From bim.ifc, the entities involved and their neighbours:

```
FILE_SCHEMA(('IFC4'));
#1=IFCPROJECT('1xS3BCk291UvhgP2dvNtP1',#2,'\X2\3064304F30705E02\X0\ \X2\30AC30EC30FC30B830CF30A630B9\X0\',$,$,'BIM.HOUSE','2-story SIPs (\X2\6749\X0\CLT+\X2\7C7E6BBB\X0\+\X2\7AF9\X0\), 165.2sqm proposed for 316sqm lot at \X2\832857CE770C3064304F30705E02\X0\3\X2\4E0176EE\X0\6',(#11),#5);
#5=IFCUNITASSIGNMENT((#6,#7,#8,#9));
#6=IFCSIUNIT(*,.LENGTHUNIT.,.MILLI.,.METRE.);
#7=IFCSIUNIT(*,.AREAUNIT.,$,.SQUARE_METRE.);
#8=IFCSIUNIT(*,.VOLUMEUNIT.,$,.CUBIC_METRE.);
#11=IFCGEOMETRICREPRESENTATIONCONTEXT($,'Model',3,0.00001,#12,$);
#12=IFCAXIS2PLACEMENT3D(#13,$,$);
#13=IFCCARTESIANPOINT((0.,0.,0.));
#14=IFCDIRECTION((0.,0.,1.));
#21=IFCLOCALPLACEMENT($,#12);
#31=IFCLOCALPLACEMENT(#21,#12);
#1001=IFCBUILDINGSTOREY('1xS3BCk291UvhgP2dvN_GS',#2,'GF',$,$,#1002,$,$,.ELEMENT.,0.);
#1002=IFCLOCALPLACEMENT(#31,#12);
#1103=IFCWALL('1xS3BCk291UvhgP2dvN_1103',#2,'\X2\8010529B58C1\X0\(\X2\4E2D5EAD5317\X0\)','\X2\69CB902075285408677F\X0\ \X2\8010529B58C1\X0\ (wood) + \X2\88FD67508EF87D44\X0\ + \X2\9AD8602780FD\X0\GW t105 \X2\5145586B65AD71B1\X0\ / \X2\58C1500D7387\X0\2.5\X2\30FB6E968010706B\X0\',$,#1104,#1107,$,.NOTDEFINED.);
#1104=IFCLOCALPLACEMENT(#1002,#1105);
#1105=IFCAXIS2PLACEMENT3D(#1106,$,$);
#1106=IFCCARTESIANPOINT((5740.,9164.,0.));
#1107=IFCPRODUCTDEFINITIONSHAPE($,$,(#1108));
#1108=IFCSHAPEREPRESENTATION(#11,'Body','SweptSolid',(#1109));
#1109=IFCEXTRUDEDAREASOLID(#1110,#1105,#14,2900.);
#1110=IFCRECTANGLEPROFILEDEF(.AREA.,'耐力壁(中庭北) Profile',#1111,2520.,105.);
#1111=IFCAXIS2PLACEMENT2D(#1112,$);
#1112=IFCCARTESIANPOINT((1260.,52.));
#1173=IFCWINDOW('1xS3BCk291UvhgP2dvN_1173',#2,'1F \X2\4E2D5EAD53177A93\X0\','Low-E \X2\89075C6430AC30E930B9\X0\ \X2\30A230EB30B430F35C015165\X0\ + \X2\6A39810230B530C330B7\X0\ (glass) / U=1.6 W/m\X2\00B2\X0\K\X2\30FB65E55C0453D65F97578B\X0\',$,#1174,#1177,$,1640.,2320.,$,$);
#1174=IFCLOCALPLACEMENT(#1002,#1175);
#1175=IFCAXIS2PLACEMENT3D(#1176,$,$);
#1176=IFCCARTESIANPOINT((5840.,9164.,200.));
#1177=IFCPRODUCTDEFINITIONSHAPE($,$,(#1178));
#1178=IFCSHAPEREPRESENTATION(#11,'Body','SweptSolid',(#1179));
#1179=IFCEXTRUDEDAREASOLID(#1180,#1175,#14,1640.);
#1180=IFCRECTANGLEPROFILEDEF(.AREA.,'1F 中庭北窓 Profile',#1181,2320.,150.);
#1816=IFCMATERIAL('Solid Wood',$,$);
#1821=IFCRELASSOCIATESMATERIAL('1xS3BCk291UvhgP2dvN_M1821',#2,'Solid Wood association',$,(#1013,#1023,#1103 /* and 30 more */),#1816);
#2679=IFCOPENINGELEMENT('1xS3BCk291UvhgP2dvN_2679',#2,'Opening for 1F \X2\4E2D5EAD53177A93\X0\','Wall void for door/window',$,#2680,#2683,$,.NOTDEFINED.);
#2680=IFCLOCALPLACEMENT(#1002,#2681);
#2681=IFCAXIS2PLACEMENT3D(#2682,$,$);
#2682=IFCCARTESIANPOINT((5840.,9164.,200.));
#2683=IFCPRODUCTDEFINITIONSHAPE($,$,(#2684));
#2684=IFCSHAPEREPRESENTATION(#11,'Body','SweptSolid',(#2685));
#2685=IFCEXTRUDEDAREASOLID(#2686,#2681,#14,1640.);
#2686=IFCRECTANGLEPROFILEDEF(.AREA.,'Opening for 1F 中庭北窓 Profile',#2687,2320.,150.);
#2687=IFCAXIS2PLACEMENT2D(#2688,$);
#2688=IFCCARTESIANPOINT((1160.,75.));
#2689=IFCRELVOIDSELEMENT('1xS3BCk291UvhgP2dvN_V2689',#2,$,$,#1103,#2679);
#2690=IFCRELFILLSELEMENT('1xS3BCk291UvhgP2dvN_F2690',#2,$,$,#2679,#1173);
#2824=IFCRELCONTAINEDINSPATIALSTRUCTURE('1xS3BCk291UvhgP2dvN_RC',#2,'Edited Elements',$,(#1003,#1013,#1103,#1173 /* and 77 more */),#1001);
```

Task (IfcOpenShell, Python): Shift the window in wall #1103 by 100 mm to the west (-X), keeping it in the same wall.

```python
import ifcopenshell
import ifcopenshell.api.geometry
import ifcopenshell.util.placement
import ifcopenshell.util.unit

model = ifcopenshell.open("bim.ifc")
unit_scale = ifcopenshell.util.unit.calculate_unit_scale(model)

window = model.by_guid("1xS3BCk291UvhgP2dvN_1173")
opening = window.FillsVoids[0].RelatingOpeningElement
wall = opening.VoidsElements[0].RelatingBuildingElement

wall_matrix = ifcopenshell.util.placement.get_local_placement(wall.ObjectPlacement)
shift = wall_matrix[:3, 0] * -0.1 / unit_scale
before = ifcopenshell.util.placement.get_local_placement(window.ObjectPlacement)[:3, 3].copy()

# The window is not placed relative to its opening, so move both.
for product in (opening, window):
    matrix = ifcopenshell.util.placement.get_local_placement(product.ObjectPlacement)
    matrix[:3, 3] += shift
    ifcopenshell.api.geometry.edit_object_placement(model, product=product, matrix=matrix, is_si=False)

after = ifcopenshell.util.placement.get_local_placement(window.ObjectPlacement)[:3, 3]
print("window moved by", (after - before).round(3) + 0.0)

model.write("bim_updated.ifc")
```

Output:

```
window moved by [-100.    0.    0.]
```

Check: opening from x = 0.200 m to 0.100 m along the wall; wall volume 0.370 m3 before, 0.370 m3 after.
